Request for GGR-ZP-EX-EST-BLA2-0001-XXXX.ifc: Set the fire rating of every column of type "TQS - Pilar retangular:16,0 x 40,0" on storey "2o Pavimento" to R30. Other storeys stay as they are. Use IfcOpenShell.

First a look at what the model holds.

```python
import ifcopenshell
import ifcopenshell.util.element

model = ifcopenshell.open("GGR-ZP-EX-EST-BLA2-0001-XXXX.ifc")
print(model.schema)
storey = next(s for s in model.by_type("IfcBuildingStorey") if s.Name == "2o Pavimento")
columns = [e for e in ifcopenshell.util.element.get_decomposition(storey) if e.is_a("IfcColumn")]
seen = {}
for e in columns:
    element_type = ifcopenshell.util.element.get_type(e)
    key = (element_type.Name if element_type != e and element_type else None, ifcopenshell.util.element.get_pset(e, "Pset_ColumnCommon", "FireRating"))
    seen[key] = seen.get(key, 0) + 1
for (name, value), count in sorted(seen.items(), key=str):
    print(count, "x", name, "|", value)
```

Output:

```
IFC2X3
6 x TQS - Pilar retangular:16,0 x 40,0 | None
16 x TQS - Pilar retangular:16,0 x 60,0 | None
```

```python
import ifcopenshell
import ifcopenshell.api.pset
import ifcopenshell.util.element

model = ifcopenshell.open("GGR-ZP-EX-EST-BLA2-0001-XXXX.ifc")

storey = next(s for s in model.by_type("IfcBuildingStorey") if s.Name == "2o Pavimento")
columns = [e for e in ifcopenshell.util.element.get_decomposition(storey) if e.is_a("IfcColumn")]

count = 0
for e in columns:
    element_type = ifcopenshell.util.element.get_type(e)
    if element_type in (None, e) or element_type.Name != "TQS - Pilar retangular:16,0 x 40,0":
        continue
    # add_pset returns the element's existing set when there is one.
    pset = ifcopenshell.api.pset.add_pset(model, product=e, name="Pset_ColumnCommon")
    ifcopenshell.api.pset.edit_pset(model, pset=pset, properties={"FireRating": "R30"})
    count += 1

print(count, "columns updated")

model.write("GGR-ZP-EX-EST-BLA2-0001-XXXX_updated.ifc")
```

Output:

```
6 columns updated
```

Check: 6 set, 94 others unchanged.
